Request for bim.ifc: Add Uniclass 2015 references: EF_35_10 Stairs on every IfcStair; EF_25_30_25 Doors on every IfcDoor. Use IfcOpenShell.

First a look at what the model holds.

```python
import ifcopenshell

model = ifcopenshell.open("bim.ifc")
print(model.schema)
print("classifications:", [c.Name for c in model.by_type("IfcClassification")])
for ifc_class in ("IfcDoor", "IfcRoof", "IfcStair", "IfcWall", "IfcWindow"):
    print(ifc_class, len(model.by_type(ifc_class)))
```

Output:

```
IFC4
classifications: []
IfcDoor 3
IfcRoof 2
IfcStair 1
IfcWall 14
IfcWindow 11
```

```python
import ifcopenshell
import ifcopenshell.api.classification

model = ifcopenshell.open("bim.ifc")

system = ifcopenshell.api.classification.add_classification(model, classification="Uniclass 2015")

codes = {
    "IfcStair": ("EF_35_10", "Stairs"),
    "IfcDoor": ("EF_25_30_25", "Doors"),
}
for ifc_class, (code, name) in codes.items():
    products = model.by_type(ifc_class)
    ifcopenshell.api.classification.add_reference(
        model, products=products, classification=system, identification=code, name=name
    )
    print(code, len(products))

model.write("bim_edited.ifc")
```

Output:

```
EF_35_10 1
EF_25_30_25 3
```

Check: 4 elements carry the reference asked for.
